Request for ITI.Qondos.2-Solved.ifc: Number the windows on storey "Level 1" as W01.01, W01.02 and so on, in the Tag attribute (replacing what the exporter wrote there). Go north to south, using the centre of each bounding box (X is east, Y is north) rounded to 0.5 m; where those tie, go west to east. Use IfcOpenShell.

First a look at what the model holds.

```python
import ifcopenshell
import ifcopenshell.util.element
import ifcopenshell.util.placement

model = ifcopenshell.open("ITI.Qondos.2-Solved.ifc")
print(model.schema)
storey = next(s for s in model.by_type("IfcBuildingStorey") if s.Name == "Level 1")
windows = [e for e in ifcopenshell.util.element.get_decomposition(storey) if e.is_a("IfcWindow")]
for e in sorted(windows, key=lambda e: e.id()):
    origin = ifcopenshell.util.placement.get_local_placement(e.ObjectPlacement)[:3, 3]
    print(e.id(), e.Tag, e.Name, origin.round(2) + 0.0, sep=" | ")
```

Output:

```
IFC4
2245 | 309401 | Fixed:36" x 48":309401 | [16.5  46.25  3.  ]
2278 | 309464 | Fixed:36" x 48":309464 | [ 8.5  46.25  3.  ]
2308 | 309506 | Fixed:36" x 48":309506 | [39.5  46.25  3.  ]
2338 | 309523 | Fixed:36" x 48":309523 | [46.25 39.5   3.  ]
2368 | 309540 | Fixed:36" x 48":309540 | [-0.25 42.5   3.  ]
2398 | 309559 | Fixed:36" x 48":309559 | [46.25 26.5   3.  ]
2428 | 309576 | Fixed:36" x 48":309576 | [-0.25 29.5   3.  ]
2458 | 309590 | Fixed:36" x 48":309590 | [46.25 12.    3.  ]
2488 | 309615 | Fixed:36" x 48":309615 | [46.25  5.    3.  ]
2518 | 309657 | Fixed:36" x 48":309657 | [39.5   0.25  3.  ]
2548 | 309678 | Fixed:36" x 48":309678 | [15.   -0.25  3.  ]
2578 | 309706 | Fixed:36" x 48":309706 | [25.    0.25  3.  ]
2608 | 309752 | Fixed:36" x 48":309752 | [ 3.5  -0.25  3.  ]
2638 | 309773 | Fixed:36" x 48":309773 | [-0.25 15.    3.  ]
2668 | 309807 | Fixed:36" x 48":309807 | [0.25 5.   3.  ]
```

```python
import ifcopenshell
import ifcopenshell.geom
import ifcopenshell.util.element
import ifcopenshell.util.shape

model = ifcopenshell.open("ITI.Qondos.2-Solved.ifc")
settings = ifcopenshell.geom.settings()
settings.set("use-world-coords", True)


def centre(element):
    shape = ifcopenshell.geom.create_shape(settings, element)
    return ifcopenshell.util.shape.get_bbox_centroid(shape.geometry)


storey = next(s for s in model.by_type("IfcBuildingStorey") if s.Name == "Level 1")
windows = [e for e in ifcopenshell.util.element.get_decomposition(storey) if e.is_a("IfcWindow")]

# Insertion points can sit at a corner or the storey origin, so sort by the geometry (in metres).
centres = {e: centre(e) for e in windows}
windows.sort(key=lambda e: (-round(centres[e][1] / 0.5), centres[e][0]))

for i, e in enumerate(windows, start=1):
    number = f"W01.{i:02d}"
    e.Tag = number
    print(e.id(), number)

model.write("ITI.Qondos.2-Solved_edited.ifc")
```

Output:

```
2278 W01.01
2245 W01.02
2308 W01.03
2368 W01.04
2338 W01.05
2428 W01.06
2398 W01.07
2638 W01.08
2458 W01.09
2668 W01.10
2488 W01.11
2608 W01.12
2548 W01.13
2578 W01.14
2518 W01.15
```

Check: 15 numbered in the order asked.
